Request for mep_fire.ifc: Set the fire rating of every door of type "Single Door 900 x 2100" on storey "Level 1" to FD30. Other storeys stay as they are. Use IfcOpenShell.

First a look at what the model holds.

```python
import ifcopenshell
import ifcopenshell.util.element

model = ifcopenshell.open("mep_fire.ifc")
print(model.schema)
storey = next(s for s in model.by_type("IfcBuildingStorey") if s.Name == "Level 1")
doors = [e for e in ifcopenshell.util.element.get_decomposition(storey) if e.is_a("IfcDoor")]
seen = {}
for e in doors:
    element_type = ifcopenshell.util.element.get_type(e)
    key = (element_type.Name if element_type != e and element_type else None, ifcopenshell.util.element.get_pset(e, "Pset_DoorCommon", "FireRating"))
    seen[key] = seen.get(key, 0) + 1
for (name, value), count in sorted(seen.items(), key=str):
    print(count, "x", name, "|", value)
```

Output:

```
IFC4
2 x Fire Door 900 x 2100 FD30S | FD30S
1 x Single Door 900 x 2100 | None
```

```python
import ifcopenshell
import ifcopenshell.api.pset
import ifcopenshell.util.element

model = ifcopenshell.open("mep_fire.ifc")

storey = next(s for s in model.by_type("IfcBuildingStorey") if s.Name == "Level 1")
doors = [e for e in ifcopenshell.util.element.get_decomposition(storey) if e.is_a("IfcDoor")]

count = 0
for e in doors:
    element_type = ifcopenshell.util.element.get_type(e)
    if element_type in (None, e) or element_type.Name != "Single Door 900 x 2100":
        continue
    # add_pset returns the element's existing set when there is one.
    pset = ifcopenshell.api.pset.add_pset(model, product=e, name="Pset_DoorCommon")
    ifcopenshell.api.pset.edit_pset(model, pset=pset, properties={"FireRating": "FD30"})
    count += 1

print(count, "doors updated")

model.write("mep_fire_updated.ifc")
```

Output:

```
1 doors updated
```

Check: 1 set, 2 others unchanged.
